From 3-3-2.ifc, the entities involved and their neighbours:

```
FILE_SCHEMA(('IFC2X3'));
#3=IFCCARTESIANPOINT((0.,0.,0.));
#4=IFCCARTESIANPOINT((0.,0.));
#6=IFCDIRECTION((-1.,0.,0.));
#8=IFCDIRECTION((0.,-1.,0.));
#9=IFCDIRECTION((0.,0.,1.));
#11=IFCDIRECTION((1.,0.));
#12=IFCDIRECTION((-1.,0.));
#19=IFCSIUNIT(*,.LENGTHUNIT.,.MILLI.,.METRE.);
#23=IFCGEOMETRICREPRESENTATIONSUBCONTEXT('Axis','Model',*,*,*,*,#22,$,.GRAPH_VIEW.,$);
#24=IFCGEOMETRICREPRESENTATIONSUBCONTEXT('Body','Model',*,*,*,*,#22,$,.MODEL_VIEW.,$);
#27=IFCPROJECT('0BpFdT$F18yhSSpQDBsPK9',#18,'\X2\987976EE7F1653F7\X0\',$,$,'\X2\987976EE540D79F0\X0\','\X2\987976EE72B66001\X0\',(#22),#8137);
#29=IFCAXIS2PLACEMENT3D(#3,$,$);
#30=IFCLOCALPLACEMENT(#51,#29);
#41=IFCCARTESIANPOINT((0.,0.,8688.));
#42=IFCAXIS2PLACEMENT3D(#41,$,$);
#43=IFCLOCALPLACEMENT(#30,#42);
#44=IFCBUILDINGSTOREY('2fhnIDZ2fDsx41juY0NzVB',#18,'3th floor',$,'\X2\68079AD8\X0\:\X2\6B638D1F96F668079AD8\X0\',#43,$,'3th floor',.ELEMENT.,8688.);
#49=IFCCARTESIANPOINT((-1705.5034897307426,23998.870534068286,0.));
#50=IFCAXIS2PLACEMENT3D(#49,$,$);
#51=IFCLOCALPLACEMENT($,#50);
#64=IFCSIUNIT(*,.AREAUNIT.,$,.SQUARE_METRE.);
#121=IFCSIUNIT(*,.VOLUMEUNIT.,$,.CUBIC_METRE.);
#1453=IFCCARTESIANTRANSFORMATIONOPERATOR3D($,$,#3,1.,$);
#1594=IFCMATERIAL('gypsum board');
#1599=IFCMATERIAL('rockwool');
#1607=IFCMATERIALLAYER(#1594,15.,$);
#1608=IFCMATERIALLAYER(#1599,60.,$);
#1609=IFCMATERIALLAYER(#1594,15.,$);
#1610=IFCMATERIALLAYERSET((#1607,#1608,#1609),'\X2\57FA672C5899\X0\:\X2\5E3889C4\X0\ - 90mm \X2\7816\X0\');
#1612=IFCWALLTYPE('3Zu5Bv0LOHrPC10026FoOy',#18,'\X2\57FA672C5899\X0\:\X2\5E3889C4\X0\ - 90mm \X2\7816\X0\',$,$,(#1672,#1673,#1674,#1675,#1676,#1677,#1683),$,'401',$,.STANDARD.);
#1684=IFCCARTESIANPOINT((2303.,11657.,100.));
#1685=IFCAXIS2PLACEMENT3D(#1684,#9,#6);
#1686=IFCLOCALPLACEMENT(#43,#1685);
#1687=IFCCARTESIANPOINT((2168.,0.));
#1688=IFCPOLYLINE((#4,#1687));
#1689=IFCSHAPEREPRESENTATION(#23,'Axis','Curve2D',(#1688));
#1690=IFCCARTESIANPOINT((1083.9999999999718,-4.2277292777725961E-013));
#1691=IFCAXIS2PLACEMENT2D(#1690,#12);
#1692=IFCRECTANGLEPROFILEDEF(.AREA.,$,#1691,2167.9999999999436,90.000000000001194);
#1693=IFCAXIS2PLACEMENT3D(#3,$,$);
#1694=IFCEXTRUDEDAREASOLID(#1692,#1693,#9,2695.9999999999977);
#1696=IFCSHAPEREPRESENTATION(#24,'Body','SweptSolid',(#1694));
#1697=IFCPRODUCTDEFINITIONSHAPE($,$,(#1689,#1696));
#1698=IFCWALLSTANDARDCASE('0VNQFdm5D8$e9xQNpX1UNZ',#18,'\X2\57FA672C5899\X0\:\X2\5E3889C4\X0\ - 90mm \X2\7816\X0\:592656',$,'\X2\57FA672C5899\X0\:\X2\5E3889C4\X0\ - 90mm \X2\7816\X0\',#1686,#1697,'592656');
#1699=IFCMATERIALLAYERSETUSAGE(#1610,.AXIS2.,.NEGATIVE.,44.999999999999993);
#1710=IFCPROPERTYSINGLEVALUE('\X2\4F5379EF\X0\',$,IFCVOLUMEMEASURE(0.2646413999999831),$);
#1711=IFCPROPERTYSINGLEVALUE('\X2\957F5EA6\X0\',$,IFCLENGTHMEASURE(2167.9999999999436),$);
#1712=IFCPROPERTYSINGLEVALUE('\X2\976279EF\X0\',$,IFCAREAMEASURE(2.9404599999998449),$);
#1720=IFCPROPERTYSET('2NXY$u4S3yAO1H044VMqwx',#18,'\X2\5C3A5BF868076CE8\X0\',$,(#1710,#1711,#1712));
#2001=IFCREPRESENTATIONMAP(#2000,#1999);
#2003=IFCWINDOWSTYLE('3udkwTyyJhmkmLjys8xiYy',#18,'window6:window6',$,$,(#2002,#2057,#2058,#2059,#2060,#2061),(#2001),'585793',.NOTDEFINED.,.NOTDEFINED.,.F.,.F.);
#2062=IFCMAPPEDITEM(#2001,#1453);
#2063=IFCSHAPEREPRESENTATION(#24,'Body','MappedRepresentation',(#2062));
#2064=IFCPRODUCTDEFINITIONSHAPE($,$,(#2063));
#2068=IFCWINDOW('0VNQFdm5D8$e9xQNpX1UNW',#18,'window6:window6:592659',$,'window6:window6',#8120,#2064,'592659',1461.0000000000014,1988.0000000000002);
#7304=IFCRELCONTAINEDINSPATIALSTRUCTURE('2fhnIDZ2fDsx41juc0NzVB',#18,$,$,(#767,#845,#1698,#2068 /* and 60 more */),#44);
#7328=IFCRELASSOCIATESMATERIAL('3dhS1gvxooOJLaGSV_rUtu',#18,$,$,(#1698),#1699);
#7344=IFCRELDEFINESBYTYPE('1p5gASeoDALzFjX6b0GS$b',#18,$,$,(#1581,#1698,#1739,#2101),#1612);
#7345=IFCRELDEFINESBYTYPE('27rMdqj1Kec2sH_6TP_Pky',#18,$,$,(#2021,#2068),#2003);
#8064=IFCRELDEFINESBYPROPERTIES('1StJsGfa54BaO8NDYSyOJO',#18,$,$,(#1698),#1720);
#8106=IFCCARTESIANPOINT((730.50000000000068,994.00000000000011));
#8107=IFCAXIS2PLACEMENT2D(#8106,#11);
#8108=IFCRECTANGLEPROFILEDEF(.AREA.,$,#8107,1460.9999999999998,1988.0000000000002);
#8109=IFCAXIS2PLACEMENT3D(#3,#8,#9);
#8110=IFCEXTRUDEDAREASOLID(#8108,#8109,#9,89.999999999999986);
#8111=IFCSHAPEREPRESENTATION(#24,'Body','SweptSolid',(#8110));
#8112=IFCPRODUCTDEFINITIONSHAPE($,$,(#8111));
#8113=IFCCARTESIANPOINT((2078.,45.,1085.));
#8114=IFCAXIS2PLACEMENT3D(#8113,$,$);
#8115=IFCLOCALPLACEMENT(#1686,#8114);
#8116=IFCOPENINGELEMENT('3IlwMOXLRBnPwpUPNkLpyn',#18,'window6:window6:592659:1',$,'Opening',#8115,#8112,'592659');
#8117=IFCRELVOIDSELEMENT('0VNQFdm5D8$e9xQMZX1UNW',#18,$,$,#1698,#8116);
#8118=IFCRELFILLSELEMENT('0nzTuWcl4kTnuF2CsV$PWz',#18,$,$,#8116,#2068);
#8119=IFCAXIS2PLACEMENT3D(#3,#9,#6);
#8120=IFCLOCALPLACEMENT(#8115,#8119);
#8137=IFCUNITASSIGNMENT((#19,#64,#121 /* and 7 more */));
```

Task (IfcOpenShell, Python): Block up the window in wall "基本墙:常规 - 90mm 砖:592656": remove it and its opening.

```python
import ifcopenshell
import ifcopenshell.api.feature
import ifcopenshell.api.pset
import ifcopenshell.api.root
import ifcopenshell.geom
import ifcopenshell.util.element
import ifcopenshell.util.shape
import ifcopenshell.util.unit

model = ifcopenshell.open("3-3-2.ifc")
area_scale = ifcopenshell.util.unit.calculate_unit_scale(model, "AREAUNIT")
volume_scale = ifcopenshell.util.unit.calculate_unit_scale(model, "VOLUMEUNIT")
settings = ifcopenshell.geom.settings()


def volume(element):
    """Net volume in cubic metres, openings subtracted."""
    shape = ifcopenshell.geom.create_shape(settings, element)
    return ifcopenshell.util.shape.get_volume(shape.geometry)


window = model.by_guid("0VNQFdm5D8$e9xQNpX1UNW")
opening = window.FillsVoids[0].RelatingOpeningElement
wall = opening.VoidsElements[0].RelatingBuildingElement
before = volume(wall)

ifcopenshell.api.root.remove_product(model, product=window)
ifcopenshell.api.feature.remove_feature(model, feature=opening)

after = volume(wall)
thickness = 0.09  # wall thickness in metres

# Update the wall's stored quantities.
pset = model.by_id(ifcopenshell.util.element.get_pset(wall, "尺寸标注", should_inherit=False)["id"])
ifcopenshell.api.pset.edit_pset(model, pset=pset, properties={
    "体积": model.create_entity("IfcVolumeMeasure", after / volume_scale),
    "面积": model.create_entity("IfcAreaMeasure", after / thickness / area_scale),
})

print(f"wall volume {before:.3f} -> {after:.3f} m3")

model.write("3-3-2_edited.ifc")
```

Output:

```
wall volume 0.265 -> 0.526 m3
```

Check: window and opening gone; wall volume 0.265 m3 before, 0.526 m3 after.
